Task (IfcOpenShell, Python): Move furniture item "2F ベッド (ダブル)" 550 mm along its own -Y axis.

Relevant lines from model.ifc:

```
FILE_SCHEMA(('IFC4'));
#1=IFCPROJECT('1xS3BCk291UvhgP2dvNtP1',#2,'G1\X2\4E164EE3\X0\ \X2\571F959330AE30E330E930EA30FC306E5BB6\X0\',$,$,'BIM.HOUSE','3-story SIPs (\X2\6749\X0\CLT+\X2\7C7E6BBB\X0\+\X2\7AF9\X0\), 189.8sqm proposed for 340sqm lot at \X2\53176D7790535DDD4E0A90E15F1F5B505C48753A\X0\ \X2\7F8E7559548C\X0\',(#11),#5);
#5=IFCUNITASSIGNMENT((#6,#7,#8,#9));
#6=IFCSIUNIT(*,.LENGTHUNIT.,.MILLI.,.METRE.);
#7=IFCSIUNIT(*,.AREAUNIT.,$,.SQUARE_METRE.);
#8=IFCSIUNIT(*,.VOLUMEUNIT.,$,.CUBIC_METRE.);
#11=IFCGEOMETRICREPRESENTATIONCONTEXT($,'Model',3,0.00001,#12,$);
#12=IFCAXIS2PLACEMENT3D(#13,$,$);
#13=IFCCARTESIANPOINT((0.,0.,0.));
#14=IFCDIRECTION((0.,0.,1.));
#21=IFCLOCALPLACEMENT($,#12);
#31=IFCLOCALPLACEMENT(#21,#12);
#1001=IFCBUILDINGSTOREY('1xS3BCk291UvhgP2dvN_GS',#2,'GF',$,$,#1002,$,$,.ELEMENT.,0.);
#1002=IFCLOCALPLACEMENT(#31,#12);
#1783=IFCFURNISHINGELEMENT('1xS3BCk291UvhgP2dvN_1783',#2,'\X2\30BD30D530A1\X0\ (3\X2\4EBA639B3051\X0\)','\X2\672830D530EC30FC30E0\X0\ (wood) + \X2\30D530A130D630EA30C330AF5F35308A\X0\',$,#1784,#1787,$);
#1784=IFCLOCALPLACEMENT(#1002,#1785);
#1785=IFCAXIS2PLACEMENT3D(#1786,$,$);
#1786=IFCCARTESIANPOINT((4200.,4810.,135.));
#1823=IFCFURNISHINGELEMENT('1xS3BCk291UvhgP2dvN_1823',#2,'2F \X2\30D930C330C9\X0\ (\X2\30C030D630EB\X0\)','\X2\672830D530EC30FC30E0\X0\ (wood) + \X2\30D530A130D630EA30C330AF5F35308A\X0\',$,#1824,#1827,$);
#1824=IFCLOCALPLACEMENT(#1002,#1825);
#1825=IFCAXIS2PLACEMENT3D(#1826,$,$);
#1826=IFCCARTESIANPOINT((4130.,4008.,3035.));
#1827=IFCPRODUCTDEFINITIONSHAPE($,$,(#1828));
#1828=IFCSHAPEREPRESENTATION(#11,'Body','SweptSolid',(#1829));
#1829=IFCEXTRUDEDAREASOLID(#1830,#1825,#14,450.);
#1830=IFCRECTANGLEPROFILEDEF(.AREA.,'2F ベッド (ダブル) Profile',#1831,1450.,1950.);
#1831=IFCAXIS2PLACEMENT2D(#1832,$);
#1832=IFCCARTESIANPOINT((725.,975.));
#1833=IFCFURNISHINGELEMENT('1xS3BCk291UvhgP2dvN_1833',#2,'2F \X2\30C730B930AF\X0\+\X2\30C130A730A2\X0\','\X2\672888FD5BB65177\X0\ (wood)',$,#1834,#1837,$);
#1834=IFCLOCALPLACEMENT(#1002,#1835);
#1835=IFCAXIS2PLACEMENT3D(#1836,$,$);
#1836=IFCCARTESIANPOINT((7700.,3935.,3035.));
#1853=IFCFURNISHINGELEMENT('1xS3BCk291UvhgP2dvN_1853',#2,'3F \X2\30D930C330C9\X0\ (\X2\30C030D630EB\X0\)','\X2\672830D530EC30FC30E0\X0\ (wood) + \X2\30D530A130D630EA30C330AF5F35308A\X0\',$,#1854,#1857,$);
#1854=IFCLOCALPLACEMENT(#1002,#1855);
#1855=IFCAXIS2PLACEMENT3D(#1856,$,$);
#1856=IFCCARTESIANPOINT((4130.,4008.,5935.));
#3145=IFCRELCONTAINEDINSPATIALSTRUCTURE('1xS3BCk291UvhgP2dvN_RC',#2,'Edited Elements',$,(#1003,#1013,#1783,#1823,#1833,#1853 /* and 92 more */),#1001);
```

```python
import ifcopenshell
import ifcopenshell.api.geometry
import ifcopenshell.util.placement
import ifcopenshell.util.unit

model = ifcopenshell.open("model.ifc")
unit_scale = ifcopenshell.util.unit.calculate_unit_scale(model)

item = model.by_id(1823)
matrix = ifcopenshell.util.placement.get_local_placement(item.ObjectPlacement)
matrix[:3, 3] -= matrix[:3, 1] * 0.55 / unit_scale
ifcopenshell.api.geometry.edit_object_placement(model, product=item, matrix=matrix, is_si=False)

print(ifcopenshell.util.placement.get_local_placement(item.ObjectPlacement).round(3) + 0.0)

model.write("model_v2.ifc")
```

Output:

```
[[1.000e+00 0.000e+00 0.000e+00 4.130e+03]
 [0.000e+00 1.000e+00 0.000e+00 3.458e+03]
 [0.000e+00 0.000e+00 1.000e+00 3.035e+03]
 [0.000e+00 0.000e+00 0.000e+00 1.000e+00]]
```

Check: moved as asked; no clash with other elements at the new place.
